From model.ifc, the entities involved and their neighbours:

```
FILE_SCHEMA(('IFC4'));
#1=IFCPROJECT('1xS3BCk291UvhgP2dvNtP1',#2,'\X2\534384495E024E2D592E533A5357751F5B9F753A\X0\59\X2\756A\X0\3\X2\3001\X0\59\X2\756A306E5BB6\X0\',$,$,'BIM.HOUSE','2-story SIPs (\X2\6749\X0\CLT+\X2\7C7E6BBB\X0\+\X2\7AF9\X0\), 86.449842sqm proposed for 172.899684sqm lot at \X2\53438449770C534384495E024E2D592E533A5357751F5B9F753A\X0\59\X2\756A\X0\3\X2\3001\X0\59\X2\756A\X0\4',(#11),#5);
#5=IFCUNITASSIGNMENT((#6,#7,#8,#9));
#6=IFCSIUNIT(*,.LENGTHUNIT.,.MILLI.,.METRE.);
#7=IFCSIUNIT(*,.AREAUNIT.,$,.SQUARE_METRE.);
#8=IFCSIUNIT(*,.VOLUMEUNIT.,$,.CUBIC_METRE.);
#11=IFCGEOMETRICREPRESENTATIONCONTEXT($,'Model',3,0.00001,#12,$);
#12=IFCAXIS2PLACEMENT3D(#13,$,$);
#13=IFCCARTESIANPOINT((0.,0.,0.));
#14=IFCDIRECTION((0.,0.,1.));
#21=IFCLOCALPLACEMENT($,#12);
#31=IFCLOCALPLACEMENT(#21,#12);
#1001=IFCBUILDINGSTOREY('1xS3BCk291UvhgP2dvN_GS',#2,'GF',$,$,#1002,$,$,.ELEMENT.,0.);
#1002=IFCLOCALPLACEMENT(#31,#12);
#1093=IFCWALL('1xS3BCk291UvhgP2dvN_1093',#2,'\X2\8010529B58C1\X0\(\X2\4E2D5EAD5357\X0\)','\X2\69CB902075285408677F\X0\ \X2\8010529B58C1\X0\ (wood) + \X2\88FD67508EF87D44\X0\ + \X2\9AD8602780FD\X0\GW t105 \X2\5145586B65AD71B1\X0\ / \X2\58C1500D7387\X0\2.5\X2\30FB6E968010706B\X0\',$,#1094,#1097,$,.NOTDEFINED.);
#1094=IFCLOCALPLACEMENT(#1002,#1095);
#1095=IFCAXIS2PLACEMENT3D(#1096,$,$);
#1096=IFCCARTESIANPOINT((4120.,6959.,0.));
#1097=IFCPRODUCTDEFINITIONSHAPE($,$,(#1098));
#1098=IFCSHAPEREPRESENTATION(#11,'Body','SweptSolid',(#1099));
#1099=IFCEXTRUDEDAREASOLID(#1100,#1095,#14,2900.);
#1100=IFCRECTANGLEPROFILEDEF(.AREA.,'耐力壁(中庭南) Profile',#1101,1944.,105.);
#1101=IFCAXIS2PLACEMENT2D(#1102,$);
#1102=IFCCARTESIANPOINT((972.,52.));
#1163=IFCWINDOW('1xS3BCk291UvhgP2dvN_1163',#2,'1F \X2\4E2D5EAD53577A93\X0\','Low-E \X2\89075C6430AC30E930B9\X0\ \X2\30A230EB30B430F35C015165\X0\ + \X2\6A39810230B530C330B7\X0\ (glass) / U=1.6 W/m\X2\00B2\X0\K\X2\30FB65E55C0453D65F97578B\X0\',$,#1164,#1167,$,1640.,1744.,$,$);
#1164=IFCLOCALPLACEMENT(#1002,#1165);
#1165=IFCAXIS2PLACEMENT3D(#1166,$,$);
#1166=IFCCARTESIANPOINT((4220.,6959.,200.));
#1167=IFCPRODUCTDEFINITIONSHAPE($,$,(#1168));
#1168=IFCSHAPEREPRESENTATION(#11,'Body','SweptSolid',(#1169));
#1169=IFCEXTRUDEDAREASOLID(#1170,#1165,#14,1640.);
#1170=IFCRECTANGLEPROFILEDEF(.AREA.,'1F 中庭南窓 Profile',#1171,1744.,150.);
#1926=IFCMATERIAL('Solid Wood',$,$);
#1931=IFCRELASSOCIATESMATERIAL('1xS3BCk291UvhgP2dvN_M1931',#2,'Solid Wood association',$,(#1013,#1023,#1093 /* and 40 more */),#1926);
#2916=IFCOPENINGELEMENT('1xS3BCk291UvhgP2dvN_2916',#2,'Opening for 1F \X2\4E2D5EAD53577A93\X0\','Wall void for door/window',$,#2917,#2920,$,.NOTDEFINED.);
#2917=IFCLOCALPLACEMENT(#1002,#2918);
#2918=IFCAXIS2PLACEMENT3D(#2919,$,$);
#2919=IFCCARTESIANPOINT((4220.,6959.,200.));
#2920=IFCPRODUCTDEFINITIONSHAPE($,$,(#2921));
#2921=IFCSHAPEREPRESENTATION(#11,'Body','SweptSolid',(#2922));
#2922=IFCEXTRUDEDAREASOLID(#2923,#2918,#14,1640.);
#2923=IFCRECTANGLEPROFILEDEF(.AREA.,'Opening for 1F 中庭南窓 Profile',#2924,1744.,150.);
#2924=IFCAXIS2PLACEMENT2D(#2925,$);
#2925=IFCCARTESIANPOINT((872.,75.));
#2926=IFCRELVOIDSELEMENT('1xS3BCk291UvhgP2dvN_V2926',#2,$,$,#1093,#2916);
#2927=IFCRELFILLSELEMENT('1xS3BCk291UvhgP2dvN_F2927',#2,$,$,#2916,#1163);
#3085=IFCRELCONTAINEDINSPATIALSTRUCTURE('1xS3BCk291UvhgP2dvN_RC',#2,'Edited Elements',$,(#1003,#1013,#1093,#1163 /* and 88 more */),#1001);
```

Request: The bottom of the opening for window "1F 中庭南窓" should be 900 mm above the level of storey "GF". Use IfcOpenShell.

```python
import numpy as np
import ifcopenshell
import ifcopenshell.api.geometry
import ifcopenshell.geom
import ifcopenshell.util.element
import ifcopenshell.util.placement
import ifcopenshell.util.shape
import ifcopenshell.util.unit

model = ifcopenshell.open("model.ifc")
unit_scale = ifcopenshell.util.unit.calculate_unit_scale(model)

window = model.by_guid("1xS3BCk291UvhgP2dvN_1163")
opening = window.FillsVoids[0].RelatingOpeningElement
storey = ifcopenshell.util.element.get_container(window, ifc_class="IfcBuildingStorey")
level = ifcopenshell.util.placement.get_local_placement(storey.ObjectPlacement)[2, 3]

# The opening's origin need not be at the sill, so measure its lowest point.
shape = ifcopenshell.geom.create_shape(ifcopenshell.geom.settings(), opening)
bottom = ifcopenshell.util.shape.get_shape_bottom_elevation(shape, shape.geometry) / unit_scale
dz = level + 0.9 / unit_scale - bottom

shift = np.array([0.0, 0.0, dz])
# The window is not placed relative to its opening, so move both.
for product in (opening, window):
    matrix = ifcopenshell.util.placement.get_local_placement(product.ObjectPlacement)
    matrix[:3, 3] += shift
    ifcopenshell.api.geometry.edit_object_placement(model, product=product, matrix=matrix, is_si=False)

print(f"moved by {dz * unit_scale:+.3f} m")

model.write("model_v2.ifc")
```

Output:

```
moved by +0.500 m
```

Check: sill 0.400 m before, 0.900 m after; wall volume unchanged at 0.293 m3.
